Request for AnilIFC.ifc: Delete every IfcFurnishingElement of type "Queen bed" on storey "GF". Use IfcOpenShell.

First a look at what the model holds.

```python
import ifcopenshell
import ifcopenshell.util.element

model = ifcopenshell.open("AnilIFC.ifc")
print(model.schema)
storey = next(s for s in model.by_type("IfcBuildingStorey") if s.Name == "GF")
furniture = [e for e in ifcopenshell.util.element.get_decomposition(storey) if e.is_a("IfcFurnishingElement")]
seen = {}
for e in furniture:
    element_type = ifcopenshell.util.element.get_type(e)
    name = element_type.Name if element_type not in (None, e) else None
    seen[name] = seen.get(name, 0) + 1
for name, count in sorted(seen.items(), key=str):
    print(count, "x", name)
```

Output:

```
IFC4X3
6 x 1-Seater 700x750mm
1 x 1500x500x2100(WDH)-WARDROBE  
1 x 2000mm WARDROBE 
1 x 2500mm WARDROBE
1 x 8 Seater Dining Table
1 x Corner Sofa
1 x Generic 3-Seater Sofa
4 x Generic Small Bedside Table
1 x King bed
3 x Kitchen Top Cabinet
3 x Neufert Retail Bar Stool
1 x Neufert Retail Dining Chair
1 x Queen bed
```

```python
import ifcopenshell
import ifcopenshell.api.root
import ifcopenshell.util.element

model = ifcopenshell.open("AnilIFC.ifc")

storey = next(s for s in model.by_type("IfcBuildingStorey") if s.Name == "GF")
furniture = [e for e in ifcopenshell.util.element.get_decomposition(storey) if e.is_a("IfcFurnishingElement")]
targets = [e for e in furniture if (t := ifcopenshell.util.element.get_type(e)) not in (None, e) and t.Name == "Queen bed"]

for e in targets:
    ifcopenshell.api.root.remove_product(model, product=e)
print(len(targets), "removed")

model.write("AnilIFC_v2.ifc")
```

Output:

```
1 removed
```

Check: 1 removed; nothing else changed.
